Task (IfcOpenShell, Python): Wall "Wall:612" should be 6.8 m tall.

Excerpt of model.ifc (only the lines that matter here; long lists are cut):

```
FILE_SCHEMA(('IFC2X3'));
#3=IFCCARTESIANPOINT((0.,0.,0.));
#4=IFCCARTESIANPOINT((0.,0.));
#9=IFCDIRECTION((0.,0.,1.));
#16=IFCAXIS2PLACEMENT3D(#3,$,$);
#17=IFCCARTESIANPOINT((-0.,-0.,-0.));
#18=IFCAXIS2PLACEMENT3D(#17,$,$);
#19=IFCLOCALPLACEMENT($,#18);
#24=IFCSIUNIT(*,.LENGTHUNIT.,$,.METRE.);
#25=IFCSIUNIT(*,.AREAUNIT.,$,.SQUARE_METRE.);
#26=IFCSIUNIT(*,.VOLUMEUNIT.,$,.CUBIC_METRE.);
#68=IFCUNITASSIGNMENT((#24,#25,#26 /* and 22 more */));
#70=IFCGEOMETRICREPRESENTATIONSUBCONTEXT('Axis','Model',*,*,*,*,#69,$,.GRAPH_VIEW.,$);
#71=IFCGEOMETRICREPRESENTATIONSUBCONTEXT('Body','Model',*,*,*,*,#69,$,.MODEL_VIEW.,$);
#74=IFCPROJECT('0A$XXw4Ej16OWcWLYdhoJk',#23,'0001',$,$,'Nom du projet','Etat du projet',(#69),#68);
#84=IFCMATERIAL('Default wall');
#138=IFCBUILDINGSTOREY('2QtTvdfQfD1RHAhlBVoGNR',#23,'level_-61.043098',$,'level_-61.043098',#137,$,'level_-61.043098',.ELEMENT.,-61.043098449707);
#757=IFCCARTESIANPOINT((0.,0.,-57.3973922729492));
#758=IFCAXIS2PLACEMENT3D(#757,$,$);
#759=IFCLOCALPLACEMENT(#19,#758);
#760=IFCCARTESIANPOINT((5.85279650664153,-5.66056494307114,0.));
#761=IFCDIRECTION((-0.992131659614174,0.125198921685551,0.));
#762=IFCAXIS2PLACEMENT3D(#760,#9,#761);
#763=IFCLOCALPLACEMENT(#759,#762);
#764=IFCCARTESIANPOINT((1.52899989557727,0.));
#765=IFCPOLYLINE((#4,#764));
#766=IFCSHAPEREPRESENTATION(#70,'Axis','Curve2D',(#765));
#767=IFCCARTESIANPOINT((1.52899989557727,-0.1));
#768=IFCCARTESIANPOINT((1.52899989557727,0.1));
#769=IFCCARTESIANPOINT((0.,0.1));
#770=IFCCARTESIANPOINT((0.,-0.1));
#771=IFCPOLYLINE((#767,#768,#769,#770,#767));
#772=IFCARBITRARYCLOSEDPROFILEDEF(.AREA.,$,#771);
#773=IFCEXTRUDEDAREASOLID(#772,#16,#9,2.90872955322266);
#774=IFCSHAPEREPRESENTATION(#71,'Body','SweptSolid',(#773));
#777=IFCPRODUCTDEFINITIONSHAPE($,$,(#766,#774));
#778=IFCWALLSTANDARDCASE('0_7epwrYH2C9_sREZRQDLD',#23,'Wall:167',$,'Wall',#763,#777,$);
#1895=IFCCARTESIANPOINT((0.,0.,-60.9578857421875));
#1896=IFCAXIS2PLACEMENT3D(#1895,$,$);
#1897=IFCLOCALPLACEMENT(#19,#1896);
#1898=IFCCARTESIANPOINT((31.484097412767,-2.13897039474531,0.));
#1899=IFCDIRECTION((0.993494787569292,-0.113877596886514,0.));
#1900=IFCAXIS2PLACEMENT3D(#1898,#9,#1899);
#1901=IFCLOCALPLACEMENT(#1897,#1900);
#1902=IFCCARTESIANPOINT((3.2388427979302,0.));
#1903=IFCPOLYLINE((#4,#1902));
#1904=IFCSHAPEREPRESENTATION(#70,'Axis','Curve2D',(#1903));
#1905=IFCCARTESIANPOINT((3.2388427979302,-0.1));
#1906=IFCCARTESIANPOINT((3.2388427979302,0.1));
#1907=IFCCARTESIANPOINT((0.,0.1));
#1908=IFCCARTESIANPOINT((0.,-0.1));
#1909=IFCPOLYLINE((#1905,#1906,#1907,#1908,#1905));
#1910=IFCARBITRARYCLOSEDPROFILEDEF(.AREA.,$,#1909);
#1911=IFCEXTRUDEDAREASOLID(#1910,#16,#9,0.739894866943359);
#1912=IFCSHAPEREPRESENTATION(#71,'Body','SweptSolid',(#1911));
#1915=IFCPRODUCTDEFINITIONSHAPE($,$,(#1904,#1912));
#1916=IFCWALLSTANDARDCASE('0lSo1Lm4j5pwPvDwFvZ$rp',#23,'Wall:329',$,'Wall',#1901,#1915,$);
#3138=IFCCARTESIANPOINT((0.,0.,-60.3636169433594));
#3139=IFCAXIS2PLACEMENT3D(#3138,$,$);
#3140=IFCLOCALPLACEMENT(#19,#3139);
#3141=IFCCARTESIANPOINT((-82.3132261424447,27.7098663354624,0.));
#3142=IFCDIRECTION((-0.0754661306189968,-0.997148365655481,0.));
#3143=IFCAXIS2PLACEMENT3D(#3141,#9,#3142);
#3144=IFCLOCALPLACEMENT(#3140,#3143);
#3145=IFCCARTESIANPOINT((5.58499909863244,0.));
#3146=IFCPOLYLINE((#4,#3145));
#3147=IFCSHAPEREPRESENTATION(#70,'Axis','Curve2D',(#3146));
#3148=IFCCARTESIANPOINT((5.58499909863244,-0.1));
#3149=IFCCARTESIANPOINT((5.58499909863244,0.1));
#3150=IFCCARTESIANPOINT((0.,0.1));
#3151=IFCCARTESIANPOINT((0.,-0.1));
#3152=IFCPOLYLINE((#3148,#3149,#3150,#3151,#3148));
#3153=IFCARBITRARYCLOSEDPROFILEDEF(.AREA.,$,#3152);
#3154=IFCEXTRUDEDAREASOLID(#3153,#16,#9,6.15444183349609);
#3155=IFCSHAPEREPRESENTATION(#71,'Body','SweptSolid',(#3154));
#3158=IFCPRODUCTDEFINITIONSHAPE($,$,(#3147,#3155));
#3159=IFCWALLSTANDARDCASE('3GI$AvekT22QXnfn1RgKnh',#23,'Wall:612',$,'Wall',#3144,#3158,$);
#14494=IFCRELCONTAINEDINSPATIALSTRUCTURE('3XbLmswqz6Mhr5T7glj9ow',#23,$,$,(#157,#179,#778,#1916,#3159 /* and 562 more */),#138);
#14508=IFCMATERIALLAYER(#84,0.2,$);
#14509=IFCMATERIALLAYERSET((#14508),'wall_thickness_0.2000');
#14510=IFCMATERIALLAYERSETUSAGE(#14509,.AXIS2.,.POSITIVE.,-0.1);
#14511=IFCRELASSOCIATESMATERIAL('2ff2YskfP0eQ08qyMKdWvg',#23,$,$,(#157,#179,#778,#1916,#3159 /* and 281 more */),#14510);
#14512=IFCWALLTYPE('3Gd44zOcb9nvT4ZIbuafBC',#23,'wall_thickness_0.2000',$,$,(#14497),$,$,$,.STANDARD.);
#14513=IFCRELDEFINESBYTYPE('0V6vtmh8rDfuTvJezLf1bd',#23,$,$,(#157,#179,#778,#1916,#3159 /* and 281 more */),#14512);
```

```python
import ifcopenshell
import ifcopenshell.geom
import ifcopenshell.util.representation
import ifcopenshell.util.shape
import ifcopenshell.util.unit

model = ifcopenshell.open("model.ifc")
unit_scale = ifcopenshell.util.unit.calculate_unit_scale(model)
settings = ifcopenshell.geom.settings()


def volume(element):
    """Net volume in cubic metres, openings subtracted."""
    shape = ifcopenshell.geom.create_shape(settings, element)
    return ifcopenshell.util.shape.get_volume(shape.geometry)


wall = model.by_id(3159)
before = volume(wall)

body = ifcopenshell.util.representation.get_representation(wall, "Model", "Body")
solid = body.Items[0]
old_height = solid.Depth
solid.Depth = 6.8 / unit_scale
after = volume(wall)

print(f"height {old_height:g} -> {solid.Depth:g}, volume {before:.3f} -> {after:.3f} m3")

model.write("model_rev.ifc")
```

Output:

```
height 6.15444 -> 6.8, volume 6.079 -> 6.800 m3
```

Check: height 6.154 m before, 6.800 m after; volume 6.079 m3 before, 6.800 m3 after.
